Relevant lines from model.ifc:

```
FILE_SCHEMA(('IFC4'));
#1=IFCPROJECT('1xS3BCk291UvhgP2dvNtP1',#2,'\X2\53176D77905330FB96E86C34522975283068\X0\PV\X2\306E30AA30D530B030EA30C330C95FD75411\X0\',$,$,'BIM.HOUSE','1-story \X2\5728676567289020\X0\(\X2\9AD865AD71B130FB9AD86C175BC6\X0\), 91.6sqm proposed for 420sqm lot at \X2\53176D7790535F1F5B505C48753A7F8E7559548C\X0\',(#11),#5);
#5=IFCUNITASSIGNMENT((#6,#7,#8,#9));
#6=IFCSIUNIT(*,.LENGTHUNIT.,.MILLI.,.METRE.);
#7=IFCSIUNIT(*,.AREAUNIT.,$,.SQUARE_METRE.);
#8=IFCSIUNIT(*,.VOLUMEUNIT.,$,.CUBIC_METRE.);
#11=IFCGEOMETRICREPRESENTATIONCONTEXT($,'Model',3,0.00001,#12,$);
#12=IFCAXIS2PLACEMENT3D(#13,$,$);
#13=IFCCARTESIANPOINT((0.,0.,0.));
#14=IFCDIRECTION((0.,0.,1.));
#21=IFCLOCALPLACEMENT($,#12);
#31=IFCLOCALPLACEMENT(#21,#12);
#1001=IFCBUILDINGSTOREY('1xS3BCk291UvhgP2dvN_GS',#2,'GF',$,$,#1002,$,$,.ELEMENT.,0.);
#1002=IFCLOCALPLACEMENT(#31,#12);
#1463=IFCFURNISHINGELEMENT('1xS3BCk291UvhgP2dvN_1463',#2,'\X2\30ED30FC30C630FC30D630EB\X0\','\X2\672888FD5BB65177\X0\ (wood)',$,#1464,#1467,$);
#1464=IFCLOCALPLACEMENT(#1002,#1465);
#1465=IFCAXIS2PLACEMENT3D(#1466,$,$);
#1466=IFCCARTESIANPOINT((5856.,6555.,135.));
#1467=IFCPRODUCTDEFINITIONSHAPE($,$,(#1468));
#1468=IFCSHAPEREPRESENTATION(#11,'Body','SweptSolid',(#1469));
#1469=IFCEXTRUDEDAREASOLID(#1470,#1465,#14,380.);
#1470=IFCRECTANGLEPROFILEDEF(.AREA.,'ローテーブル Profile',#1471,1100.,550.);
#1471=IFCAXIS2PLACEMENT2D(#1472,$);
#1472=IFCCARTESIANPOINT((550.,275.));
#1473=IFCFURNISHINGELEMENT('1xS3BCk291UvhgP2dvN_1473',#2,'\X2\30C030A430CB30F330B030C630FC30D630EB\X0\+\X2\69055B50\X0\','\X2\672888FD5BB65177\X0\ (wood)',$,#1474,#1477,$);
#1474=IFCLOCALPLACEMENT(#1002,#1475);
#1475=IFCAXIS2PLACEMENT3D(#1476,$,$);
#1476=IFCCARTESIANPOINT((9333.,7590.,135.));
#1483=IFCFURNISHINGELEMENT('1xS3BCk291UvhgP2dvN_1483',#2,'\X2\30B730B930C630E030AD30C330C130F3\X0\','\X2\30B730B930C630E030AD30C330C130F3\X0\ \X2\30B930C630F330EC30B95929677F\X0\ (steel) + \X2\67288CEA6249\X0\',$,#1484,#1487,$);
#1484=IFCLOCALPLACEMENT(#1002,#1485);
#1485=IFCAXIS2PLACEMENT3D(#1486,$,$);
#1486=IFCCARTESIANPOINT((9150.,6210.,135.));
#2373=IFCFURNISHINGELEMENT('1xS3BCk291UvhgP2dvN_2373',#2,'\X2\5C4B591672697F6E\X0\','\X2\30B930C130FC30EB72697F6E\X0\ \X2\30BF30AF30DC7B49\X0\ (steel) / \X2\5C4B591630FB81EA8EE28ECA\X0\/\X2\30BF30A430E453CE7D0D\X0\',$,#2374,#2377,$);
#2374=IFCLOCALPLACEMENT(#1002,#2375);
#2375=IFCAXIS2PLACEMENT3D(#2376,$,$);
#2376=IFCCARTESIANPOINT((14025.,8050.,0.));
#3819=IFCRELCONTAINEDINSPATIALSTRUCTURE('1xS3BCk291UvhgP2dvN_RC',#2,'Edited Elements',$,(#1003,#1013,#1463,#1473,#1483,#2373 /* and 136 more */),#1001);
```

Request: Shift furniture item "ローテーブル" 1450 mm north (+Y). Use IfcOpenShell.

```python
import ifcopenshell
import ifcopenshell.api.geometry
import ifcopenshell.util.placement

model = ifcopenshell.open("model.ifc")

item = model.by_guid("1xS3BCk291UvhgP2dvN_1463")
matrix = ifcopenshell.util.placement.get_local_placement(item.ObjectPlacement)
matrix[1, 3] += 1450.0
ifcopenshell.api.geometry.edit_object_placement(model, product=item, matrix=matrix, is_si=False)

print(ifcopenshell.util.placement.get_local_placement(item.ObjectPlacement).round(3) + 0.0)

model.write("model_edited.ifc")
```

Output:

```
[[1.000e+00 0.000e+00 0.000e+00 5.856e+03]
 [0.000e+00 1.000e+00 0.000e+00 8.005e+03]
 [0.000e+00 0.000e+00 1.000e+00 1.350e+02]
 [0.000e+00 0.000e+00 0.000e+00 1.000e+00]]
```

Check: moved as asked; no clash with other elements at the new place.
